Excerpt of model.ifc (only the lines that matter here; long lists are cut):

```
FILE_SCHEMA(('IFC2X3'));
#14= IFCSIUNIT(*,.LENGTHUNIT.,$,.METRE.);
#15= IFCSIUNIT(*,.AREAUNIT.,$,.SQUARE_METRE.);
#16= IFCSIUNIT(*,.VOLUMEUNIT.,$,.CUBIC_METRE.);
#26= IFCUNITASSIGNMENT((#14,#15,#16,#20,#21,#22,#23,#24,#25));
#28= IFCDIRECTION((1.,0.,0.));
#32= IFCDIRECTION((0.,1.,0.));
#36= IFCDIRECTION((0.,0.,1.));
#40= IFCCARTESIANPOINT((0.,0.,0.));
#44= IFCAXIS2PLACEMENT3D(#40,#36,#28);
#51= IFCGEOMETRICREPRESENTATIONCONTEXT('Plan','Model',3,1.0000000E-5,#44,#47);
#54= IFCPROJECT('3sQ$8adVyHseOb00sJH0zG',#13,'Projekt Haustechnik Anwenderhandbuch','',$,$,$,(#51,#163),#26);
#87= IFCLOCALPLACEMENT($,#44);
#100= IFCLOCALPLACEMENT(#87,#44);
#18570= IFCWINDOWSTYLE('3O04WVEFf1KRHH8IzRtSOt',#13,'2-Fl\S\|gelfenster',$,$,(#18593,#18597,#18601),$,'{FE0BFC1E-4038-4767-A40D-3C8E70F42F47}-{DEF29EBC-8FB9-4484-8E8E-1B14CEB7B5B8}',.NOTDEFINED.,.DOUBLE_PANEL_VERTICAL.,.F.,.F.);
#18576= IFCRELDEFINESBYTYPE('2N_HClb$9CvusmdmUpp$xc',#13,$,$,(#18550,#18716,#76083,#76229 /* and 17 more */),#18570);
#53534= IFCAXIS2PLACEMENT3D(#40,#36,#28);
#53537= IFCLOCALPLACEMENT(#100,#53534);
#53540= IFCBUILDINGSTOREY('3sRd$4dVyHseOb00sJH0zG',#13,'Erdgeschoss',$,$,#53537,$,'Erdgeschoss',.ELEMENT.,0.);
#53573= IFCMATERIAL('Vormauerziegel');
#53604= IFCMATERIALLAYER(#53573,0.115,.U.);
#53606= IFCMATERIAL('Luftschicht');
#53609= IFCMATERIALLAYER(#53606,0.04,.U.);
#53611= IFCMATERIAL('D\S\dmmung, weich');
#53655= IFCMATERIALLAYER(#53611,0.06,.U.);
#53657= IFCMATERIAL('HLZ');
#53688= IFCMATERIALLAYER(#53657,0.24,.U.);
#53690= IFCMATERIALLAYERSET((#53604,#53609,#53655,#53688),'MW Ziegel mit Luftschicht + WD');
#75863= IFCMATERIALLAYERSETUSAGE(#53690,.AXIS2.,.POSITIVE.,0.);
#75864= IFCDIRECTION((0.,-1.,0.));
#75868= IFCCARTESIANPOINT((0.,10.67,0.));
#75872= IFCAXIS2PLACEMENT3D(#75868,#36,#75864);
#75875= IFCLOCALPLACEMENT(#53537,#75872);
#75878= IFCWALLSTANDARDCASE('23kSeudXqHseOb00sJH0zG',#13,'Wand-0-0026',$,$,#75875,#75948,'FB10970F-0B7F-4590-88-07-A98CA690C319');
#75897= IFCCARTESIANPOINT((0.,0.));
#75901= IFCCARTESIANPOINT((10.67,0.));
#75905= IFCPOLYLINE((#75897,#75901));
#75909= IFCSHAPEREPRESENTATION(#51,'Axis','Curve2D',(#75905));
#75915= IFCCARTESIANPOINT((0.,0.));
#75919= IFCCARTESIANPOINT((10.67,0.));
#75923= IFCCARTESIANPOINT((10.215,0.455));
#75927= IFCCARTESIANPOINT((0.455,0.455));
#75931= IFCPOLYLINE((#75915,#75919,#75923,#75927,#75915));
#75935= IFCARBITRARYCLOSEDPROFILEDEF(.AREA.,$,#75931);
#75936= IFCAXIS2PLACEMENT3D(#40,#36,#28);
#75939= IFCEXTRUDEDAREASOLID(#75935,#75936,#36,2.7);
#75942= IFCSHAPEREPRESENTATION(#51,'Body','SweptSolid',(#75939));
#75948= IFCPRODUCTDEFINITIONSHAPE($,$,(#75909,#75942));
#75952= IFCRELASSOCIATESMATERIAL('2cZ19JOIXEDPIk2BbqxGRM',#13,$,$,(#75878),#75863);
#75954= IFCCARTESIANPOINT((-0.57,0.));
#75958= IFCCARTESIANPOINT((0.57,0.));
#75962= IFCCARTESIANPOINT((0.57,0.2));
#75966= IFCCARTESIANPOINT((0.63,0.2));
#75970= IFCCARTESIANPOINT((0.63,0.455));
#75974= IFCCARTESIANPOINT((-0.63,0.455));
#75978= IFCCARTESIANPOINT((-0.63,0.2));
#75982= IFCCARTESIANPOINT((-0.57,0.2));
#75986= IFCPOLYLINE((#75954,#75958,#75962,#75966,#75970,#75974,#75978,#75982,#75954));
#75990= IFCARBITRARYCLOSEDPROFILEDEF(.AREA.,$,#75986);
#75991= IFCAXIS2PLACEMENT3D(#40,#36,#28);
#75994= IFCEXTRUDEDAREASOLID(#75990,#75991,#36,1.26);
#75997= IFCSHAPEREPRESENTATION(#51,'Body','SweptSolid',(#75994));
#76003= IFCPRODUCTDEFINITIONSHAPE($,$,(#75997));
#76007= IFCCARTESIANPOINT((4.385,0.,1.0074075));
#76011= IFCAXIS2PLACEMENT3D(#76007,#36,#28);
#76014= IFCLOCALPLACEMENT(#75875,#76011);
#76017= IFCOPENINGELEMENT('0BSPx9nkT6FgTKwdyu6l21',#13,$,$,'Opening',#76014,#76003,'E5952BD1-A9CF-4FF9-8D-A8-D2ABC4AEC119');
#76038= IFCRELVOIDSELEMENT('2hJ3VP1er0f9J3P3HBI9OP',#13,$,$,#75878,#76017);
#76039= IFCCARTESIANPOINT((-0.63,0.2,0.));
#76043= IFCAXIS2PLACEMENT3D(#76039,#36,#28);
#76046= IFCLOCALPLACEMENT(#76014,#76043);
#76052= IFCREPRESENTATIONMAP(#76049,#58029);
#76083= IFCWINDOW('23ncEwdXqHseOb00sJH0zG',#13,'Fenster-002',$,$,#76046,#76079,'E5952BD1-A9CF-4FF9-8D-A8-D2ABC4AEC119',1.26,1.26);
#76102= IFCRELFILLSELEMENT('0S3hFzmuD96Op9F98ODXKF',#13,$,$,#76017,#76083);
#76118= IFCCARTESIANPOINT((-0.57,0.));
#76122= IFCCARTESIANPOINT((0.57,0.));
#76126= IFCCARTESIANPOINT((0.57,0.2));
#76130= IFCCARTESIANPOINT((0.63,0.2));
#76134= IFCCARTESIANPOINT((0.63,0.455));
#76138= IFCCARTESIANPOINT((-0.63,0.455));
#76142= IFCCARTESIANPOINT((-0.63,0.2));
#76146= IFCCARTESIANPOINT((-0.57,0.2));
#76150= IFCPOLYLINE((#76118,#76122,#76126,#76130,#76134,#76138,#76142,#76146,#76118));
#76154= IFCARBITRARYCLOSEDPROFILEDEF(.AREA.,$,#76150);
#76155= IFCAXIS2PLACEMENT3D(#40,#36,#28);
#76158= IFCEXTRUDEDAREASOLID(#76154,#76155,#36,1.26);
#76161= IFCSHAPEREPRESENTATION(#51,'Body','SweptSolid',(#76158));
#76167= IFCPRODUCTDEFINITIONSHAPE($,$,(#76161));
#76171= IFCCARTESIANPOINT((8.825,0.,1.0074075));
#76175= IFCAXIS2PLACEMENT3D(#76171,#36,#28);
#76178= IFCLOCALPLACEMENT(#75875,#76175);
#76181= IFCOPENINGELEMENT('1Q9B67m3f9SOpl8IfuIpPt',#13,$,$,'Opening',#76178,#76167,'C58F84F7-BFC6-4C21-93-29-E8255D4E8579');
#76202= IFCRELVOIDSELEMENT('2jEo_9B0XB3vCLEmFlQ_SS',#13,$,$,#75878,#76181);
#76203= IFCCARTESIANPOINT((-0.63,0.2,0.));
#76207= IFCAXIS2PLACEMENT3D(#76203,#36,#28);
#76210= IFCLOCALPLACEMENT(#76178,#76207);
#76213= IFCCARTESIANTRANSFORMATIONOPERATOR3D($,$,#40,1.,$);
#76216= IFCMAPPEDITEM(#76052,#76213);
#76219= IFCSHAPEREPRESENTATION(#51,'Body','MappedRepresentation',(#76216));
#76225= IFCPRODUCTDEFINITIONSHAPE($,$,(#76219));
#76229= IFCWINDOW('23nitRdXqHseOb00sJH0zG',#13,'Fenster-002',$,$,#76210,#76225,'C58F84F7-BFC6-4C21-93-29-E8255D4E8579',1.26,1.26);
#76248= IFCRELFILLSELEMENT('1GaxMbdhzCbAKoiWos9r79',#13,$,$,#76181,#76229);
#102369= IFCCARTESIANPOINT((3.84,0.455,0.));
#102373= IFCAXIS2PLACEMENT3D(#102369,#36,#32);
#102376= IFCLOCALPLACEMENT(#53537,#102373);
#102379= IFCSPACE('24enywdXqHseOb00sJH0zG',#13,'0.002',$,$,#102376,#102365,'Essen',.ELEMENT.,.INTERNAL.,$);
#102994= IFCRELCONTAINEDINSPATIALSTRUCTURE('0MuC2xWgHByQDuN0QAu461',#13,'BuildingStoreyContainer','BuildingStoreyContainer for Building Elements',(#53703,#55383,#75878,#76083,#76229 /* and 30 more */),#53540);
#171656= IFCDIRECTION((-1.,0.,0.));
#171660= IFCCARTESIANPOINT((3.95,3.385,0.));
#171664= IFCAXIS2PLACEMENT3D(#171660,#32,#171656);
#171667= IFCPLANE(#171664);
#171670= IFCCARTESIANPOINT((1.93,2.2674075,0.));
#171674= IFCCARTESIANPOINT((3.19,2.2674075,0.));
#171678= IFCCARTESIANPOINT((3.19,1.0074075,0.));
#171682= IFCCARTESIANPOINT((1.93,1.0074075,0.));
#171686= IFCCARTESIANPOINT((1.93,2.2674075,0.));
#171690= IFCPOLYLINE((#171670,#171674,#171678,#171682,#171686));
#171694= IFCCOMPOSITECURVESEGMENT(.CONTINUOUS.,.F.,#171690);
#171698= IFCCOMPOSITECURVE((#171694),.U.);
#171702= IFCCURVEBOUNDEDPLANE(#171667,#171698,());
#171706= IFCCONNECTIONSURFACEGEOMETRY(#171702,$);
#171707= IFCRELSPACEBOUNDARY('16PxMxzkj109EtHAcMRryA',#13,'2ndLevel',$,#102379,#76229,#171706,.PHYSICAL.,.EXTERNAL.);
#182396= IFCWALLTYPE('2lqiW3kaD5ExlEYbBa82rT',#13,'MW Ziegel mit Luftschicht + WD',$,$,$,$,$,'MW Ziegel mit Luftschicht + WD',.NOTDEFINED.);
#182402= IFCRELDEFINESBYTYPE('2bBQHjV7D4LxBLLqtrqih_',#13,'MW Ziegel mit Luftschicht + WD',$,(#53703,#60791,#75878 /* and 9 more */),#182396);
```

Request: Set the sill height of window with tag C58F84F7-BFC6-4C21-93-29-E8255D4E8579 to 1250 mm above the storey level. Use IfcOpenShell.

```python
import numpy as np
import ifcopenshell
import ifcopenshell.api.geometry
import ifcopenshell.geom
import ifcopenshell.util.element
import ifcopenshell.util.placement
import ifcopenshell.util.shape
import ifcopenshell.util.unit

model = ifcopenshell.open("model.ifc")
unit_scale = ifcopenshell.util.unit.calculate_unit_scale(model)

window = model.by_guid("23nitRdXqHseOb00sJH0zG")
opening = window.FillsVoids[0].RelatingOpeningElement
storey = ifcopenshell.util.element.get_container(window, ifc_class="IfcBuildingStorey")
level = ifcopenshell.util.placement.get_local_placement(storey.ObjectPlacement)[2, 3]

# The opening's origin need not be at the sill, so measure its lowest point.
shape = ifcopenshell.geom.create_shape(ifcopenshell.geom.settings(), opening)
bottom = ifcopenshell.util.shape.get_shape_bottom_elevation(shape, shape.geometry) / unit_scale
dz = level + 1.25 - bottom

shift = np.array([0.0, 0.0, dz])
# The window is placed relative to its opening, so it follows when the opening moves.
matrix = ifcopenshell.util.placement.get_local_placement(opening.ObjectPlacement)
matrix[:3, 3] += shift
ifcopenshell.api.geometry.edit_object_placement(
    model, product=opening, matrix=matrix, is_si=False, should_transform_children=True
)

# Space boundary surfaces are stored in each space's coordinates; move them too.
for rel in window.ProvidesBoundaries:
    if not rel.ConnectionGeometry:
        continue
    surface = rel.ConnectionGeometry.SurfaceOnRelatingElement.BasisSurface
    space_matrix = ifcopenshell.util.placement.get_local_placement(rel.RelatingSpace.ObjectPlacement)
    point = np.array(surface.Position.Location.Coordinates) + space_matrix[:3, :3].T @ shift
    surface.Position = model.createIfcAxis2Placement3D(
        model.createIfcCartesianPoint(point.tolist()), surface.Position.Axis, surface.Position.RefDirection
    )

print(f"moved by {dz * unit_scale:+.3f} m")

model.write("model_v2.ifc")
```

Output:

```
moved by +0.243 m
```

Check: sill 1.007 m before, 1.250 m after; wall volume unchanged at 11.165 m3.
